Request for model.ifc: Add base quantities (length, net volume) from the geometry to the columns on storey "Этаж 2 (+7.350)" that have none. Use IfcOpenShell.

First a look at what the model holds.

```python
import ifcopenshell
import ifcopenshell.util.element
import ifcopenshell.util.unit

model = ifcopenshell.open("model.ifc")
print(model.schema)
for unit_type in ("LENGTHUNIT", "AREAUNIT", "VOLUMEUNIT"):
    print(unit_type, ifcopenshell.util.unit.calculate_unit_scale(model, unit_type))
storey = next(s for s in model.by_type("IfcBuildingStorey") if s.Name == "Этаж 2 (+7.350)")
columns = [e for e in ifcopenshell.util.element.get_decomposition(storey) if e.is_a("IfcColumn")]
for e in sorted(columns, key=lambda e: e.id()):
    print(e.id(), e.is_a(), e.Name, list(ifcopenshell.util.element.get_psets(e, qtos_only=True)), sep=" | ")
```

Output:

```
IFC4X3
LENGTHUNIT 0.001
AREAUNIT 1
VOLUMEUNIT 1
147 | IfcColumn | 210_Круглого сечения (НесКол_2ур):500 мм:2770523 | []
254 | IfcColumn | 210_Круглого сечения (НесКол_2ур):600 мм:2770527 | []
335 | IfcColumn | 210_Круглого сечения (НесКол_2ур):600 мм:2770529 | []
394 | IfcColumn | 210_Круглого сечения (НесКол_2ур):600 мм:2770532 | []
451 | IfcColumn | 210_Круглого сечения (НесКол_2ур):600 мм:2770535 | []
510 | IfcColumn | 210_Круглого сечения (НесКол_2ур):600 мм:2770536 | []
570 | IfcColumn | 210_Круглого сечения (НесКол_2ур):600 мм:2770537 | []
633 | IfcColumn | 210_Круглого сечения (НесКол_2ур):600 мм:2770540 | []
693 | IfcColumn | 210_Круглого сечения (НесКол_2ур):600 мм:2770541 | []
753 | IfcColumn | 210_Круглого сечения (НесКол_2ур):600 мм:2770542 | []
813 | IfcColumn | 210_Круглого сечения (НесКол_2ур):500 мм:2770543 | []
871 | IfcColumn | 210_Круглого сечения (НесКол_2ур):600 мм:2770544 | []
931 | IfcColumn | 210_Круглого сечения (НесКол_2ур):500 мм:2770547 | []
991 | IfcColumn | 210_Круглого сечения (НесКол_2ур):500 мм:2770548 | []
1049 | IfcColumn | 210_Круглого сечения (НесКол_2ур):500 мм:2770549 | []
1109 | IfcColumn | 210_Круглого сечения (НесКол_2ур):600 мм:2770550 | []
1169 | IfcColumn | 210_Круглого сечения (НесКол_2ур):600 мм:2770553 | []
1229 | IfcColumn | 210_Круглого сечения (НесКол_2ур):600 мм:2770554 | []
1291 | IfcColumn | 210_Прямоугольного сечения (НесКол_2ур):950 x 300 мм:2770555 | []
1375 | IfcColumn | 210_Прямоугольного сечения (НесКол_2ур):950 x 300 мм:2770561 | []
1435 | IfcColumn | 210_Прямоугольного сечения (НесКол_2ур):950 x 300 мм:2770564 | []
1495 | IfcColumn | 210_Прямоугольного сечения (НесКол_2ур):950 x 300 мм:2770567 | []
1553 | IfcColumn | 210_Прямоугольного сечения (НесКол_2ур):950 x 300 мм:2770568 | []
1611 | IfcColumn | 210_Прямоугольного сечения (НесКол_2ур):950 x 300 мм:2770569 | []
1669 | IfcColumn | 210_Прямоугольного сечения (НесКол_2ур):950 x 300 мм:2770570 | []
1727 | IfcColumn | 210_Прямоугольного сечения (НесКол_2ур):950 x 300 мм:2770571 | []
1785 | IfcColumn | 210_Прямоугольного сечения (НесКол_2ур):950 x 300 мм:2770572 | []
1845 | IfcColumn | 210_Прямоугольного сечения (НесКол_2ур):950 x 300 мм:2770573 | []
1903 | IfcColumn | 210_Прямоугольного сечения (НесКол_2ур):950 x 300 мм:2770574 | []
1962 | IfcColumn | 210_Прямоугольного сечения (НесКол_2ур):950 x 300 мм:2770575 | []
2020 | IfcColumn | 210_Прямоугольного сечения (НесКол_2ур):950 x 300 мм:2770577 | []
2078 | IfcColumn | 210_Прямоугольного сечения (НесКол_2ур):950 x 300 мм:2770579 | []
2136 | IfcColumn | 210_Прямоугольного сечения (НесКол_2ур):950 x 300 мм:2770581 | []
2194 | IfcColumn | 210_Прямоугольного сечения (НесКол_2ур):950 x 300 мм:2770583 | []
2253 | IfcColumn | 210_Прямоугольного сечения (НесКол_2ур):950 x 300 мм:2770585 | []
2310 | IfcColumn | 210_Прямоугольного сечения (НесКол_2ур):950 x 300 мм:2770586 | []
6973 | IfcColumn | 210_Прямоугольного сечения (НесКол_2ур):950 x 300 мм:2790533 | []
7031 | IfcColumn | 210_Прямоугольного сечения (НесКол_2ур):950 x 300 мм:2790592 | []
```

```python
import ifcopenshell
import ifcopenshell.api.pset
import ifcopenshell.geom
import ifcopenshell.util.element
import ifcopenshell.util.shape
import ifcopenshell.util.unit

model = ifcopenshell.open("model.ifc")
unit_scale = ifcopenshell.util.unit.calculate_unit_scale(model)
volume_scale = ifcopenshell.util.unit.calculate_unit_scale(model, "VOLUMEUNIT")
settings = ifcopenshell.geom.settings()

storey = next(s for s in model.by_type("IfcBuildingStorey") if s.Name == "Этаж 2 (+7.350)")
columns = [e for e in ifcopenshell.util.element.get_decomposition(storey) if e.is_a("IfcColumn")]

for e in sorted(columns, key=lambda e: e.id()):
    if ifcopenshell.util.element.get_psets(e, qtos_only=True, should_inherit=False):
        continue
    # Geometry comes back in metres, in the element's own axes.
    shape = ifcopenshell.geom.create_shape(settings, e)
    values = {
        "Length": ifcopenshell.util.shape.get_z(shape.geometry) / unit_scale,
        "NetVolume": ifcopenshell.util.shape.get_volume(shape.geometry) / volume_scale,
    }
    qto = ifcopenshell.api.pset.add_qto(model, product=e, name="Qto_ColumnBaseQuantities")
    ifcopenshell.api.pset.edit_qto(model, qto=qto, properties=values)
    print(e.id(), {k: round(v, 3) for k, v in values.items()})

model.write("model_edited.ifc")
```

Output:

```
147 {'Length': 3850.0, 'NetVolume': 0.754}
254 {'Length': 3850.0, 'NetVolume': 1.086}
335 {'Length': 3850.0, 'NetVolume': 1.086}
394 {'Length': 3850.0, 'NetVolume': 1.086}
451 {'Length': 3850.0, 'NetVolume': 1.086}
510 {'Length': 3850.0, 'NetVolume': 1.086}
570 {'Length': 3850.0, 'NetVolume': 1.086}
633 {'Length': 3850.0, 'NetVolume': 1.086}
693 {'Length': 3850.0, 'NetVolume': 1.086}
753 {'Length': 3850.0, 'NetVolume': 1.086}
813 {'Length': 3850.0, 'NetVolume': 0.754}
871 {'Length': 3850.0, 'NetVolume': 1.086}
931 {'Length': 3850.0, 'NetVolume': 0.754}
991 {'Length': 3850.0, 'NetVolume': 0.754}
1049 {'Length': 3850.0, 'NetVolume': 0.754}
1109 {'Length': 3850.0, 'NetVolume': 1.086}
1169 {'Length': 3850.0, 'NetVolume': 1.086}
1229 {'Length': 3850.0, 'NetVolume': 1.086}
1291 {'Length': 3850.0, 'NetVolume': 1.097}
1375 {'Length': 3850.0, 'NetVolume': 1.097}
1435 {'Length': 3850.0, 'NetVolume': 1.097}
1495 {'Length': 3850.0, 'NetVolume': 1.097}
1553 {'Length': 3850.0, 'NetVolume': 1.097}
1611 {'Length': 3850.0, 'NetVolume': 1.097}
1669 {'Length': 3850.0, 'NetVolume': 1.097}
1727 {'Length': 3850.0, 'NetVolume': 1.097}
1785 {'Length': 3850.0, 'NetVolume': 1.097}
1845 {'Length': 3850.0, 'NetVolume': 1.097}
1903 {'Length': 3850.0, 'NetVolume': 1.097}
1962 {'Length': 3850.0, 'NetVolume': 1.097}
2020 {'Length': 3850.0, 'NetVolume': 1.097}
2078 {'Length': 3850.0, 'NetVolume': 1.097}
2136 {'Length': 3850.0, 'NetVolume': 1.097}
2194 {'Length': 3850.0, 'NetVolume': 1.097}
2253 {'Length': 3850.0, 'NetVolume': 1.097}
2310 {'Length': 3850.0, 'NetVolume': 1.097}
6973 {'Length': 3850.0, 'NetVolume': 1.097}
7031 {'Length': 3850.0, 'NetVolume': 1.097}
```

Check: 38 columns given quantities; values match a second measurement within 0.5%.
